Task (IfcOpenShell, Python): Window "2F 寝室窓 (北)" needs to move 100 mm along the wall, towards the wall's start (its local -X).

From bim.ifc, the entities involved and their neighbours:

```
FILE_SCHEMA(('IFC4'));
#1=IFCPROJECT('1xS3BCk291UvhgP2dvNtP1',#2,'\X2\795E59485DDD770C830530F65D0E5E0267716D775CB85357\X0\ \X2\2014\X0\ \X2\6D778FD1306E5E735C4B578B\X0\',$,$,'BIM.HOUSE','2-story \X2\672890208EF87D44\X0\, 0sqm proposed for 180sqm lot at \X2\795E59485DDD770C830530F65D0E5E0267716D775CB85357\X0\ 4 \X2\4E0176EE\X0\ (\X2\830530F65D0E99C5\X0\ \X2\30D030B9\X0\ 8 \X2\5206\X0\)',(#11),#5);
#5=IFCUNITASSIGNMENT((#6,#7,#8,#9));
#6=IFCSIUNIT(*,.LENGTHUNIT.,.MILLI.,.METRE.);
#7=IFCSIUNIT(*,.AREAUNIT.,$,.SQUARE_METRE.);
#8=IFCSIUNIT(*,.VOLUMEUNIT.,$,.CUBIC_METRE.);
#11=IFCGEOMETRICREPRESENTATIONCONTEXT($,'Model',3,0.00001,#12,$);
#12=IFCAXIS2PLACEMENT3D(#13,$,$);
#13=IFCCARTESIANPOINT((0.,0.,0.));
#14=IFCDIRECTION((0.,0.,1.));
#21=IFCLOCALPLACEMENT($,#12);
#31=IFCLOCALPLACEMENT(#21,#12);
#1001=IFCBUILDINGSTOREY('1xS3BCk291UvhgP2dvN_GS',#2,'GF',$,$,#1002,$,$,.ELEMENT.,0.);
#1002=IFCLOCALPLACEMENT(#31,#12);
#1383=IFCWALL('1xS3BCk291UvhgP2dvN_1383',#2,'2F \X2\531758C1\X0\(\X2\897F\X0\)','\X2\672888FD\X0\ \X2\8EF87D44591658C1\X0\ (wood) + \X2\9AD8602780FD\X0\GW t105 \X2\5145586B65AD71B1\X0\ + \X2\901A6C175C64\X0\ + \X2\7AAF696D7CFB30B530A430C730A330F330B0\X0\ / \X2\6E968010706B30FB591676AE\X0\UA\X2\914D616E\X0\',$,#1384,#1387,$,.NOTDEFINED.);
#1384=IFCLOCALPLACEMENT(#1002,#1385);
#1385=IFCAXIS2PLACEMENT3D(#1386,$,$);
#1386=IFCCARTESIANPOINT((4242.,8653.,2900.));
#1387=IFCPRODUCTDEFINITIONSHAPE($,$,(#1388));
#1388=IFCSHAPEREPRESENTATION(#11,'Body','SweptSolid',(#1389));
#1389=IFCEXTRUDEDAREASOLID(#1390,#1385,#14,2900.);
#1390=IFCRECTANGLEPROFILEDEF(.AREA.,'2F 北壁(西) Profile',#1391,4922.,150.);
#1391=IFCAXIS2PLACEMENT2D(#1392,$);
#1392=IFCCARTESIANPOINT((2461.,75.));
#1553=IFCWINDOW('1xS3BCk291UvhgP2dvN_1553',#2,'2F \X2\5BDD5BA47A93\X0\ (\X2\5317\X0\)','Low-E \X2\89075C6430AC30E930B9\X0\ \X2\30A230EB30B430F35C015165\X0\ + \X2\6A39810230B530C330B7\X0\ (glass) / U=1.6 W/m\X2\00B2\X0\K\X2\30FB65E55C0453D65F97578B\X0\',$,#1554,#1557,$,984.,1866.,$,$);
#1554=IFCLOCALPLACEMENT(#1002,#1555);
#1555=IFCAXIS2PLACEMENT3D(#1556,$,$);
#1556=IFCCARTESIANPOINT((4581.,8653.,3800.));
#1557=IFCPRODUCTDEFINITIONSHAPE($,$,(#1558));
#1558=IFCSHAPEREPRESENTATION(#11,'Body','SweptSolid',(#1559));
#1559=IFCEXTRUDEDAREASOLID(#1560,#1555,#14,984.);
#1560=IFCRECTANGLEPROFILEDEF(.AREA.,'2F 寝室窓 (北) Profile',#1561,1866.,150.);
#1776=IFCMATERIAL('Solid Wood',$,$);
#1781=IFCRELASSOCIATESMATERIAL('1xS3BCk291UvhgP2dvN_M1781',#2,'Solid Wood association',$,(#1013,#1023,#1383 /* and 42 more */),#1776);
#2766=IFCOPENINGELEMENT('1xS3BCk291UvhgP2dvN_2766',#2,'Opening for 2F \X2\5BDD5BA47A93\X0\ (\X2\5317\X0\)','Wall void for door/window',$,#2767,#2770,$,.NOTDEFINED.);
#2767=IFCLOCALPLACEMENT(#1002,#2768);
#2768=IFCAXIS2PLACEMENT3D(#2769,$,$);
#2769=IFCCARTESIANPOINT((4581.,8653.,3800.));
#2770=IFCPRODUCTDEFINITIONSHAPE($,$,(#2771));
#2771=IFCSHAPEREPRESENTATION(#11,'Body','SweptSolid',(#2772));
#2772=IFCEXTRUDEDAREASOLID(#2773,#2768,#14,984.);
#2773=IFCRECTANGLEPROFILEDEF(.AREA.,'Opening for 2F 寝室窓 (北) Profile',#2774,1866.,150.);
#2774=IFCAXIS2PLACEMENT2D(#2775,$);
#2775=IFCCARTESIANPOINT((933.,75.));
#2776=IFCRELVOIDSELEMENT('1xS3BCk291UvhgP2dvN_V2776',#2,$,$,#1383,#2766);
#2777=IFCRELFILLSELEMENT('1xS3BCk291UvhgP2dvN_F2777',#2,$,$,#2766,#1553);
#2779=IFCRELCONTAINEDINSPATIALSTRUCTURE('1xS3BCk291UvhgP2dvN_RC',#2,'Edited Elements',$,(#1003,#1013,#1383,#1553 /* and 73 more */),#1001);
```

```python
import ifcopenshell
import ifcopenshell.api.geometry
import ifcopenshell.util.placement

model = ifcopenshell.open("bim.ifc")

window = model.by_guid("1xS3BCk291UvhgP2dvN_1553")
opening = window.FillsVoids[0].RelatingOpeningElement
wall = opening.VoidsElements[0].RelatingBuildingElement

wall_matrix = ifcopenshell.util.placement.get_local_placement(wall.ObjectPlacement)
shift = wall_matrix[:3, 0] * -100.0
before = ifcopenshell.util.placement.get_local_placement(window.ObjectPlacement)[:3, 3].copy()

# The window is not placed relative to its opening, so move both.
for product in (opening, window):
    matrix = ifcopenshell.util.placement.get_local_placement(product.ObjectPlacement)
    matrix[:3, 3] += shift
    ifcopenshell.api.geometry.edit_object_placement(model, product=product, matrix=matrix, is_si=False)

after = ifcopenshell.util.placement.get_local_placement(window.ObjectPlacement)[:3, 3]
print("window moved by", (after - before).round(3) + 0.0)

model.write("bim_v2.ifc")
```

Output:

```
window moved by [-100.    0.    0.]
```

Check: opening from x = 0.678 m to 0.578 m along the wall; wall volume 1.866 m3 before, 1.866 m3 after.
